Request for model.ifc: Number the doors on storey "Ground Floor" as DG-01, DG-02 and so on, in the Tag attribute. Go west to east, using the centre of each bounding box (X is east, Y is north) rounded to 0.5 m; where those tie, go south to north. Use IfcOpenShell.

First a look at what the model holds.

```python
import ifcopenshell
import ifcopenshell.util.element
import ifcopenshell.util.placement

model = ifcopenshell.open("model.ifc")
print(model.schema)
storey = next(s for s in model.by_type("IfcBuildingStorey") if s.Name == "Ground Floor")
doors = [e for e in ifcopenshell.util.element.get_decomposition(storey) if e.is_a("IfcDoor")]
for e in sorted(doors, key=lambda e: e.id()):
    origin = ifcopenshell.util.placement.get_local_placement(e.ObjectPlacement)[:3, 3]
    print(e.id(), e.Tag, e.Name, origin.round(2) + 0.0, sep=" | ")
```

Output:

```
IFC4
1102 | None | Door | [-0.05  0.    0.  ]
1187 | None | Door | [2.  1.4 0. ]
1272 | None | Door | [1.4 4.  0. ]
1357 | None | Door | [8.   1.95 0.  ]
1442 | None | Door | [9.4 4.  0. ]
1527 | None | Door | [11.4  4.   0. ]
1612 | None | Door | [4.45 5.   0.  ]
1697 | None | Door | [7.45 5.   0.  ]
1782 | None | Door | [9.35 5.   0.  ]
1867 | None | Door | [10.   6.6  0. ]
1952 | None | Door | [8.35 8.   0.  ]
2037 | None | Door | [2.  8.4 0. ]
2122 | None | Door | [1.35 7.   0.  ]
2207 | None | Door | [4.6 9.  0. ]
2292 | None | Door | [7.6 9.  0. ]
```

```python
import ifcopenshell
import ifcopenshell.geom
import ifcopenshell.util.element
import ifcopenshell.util.shape

model = ifcopenshell.open("model.ifc")
settings = ifcopenshell.geom.settings()
settings.set("use-world-coords", True)


def centre(element):
    shape = ifcopenshell.geom.create_shape(settings, element)
    return ifcopenshell.util.shape.get_bbox_centroid(shape.geometry)


storey = next(s for s in model.by_type("IfcBuildingStorey") if s.Name == "Ground Floor")
doors = [e for e in ifcopenshell.util.element.get_decomposition(storey) if e.is_a("IfcDoor")]

# Insertion points can sit at a corner or the storey origin, so sort by the geometry (in metres).
centres = {e: centre(e) for e in doors}
doors.sort(key=lambda e: (round(centres[e][0] / 0.5), centres[e][1]))

for i, e in enumerate(doors, start=1):
    number = f"DG-{i:02d}"
    e.Tag = number
    print(e.id(), number)

model.write("model-out.ifc")
```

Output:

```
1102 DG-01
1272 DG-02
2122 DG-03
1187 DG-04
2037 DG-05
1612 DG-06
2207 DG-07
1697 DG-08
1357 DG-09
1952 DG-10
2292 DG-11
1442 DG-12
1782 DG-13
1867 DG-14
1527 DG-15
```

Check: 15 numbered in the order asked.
